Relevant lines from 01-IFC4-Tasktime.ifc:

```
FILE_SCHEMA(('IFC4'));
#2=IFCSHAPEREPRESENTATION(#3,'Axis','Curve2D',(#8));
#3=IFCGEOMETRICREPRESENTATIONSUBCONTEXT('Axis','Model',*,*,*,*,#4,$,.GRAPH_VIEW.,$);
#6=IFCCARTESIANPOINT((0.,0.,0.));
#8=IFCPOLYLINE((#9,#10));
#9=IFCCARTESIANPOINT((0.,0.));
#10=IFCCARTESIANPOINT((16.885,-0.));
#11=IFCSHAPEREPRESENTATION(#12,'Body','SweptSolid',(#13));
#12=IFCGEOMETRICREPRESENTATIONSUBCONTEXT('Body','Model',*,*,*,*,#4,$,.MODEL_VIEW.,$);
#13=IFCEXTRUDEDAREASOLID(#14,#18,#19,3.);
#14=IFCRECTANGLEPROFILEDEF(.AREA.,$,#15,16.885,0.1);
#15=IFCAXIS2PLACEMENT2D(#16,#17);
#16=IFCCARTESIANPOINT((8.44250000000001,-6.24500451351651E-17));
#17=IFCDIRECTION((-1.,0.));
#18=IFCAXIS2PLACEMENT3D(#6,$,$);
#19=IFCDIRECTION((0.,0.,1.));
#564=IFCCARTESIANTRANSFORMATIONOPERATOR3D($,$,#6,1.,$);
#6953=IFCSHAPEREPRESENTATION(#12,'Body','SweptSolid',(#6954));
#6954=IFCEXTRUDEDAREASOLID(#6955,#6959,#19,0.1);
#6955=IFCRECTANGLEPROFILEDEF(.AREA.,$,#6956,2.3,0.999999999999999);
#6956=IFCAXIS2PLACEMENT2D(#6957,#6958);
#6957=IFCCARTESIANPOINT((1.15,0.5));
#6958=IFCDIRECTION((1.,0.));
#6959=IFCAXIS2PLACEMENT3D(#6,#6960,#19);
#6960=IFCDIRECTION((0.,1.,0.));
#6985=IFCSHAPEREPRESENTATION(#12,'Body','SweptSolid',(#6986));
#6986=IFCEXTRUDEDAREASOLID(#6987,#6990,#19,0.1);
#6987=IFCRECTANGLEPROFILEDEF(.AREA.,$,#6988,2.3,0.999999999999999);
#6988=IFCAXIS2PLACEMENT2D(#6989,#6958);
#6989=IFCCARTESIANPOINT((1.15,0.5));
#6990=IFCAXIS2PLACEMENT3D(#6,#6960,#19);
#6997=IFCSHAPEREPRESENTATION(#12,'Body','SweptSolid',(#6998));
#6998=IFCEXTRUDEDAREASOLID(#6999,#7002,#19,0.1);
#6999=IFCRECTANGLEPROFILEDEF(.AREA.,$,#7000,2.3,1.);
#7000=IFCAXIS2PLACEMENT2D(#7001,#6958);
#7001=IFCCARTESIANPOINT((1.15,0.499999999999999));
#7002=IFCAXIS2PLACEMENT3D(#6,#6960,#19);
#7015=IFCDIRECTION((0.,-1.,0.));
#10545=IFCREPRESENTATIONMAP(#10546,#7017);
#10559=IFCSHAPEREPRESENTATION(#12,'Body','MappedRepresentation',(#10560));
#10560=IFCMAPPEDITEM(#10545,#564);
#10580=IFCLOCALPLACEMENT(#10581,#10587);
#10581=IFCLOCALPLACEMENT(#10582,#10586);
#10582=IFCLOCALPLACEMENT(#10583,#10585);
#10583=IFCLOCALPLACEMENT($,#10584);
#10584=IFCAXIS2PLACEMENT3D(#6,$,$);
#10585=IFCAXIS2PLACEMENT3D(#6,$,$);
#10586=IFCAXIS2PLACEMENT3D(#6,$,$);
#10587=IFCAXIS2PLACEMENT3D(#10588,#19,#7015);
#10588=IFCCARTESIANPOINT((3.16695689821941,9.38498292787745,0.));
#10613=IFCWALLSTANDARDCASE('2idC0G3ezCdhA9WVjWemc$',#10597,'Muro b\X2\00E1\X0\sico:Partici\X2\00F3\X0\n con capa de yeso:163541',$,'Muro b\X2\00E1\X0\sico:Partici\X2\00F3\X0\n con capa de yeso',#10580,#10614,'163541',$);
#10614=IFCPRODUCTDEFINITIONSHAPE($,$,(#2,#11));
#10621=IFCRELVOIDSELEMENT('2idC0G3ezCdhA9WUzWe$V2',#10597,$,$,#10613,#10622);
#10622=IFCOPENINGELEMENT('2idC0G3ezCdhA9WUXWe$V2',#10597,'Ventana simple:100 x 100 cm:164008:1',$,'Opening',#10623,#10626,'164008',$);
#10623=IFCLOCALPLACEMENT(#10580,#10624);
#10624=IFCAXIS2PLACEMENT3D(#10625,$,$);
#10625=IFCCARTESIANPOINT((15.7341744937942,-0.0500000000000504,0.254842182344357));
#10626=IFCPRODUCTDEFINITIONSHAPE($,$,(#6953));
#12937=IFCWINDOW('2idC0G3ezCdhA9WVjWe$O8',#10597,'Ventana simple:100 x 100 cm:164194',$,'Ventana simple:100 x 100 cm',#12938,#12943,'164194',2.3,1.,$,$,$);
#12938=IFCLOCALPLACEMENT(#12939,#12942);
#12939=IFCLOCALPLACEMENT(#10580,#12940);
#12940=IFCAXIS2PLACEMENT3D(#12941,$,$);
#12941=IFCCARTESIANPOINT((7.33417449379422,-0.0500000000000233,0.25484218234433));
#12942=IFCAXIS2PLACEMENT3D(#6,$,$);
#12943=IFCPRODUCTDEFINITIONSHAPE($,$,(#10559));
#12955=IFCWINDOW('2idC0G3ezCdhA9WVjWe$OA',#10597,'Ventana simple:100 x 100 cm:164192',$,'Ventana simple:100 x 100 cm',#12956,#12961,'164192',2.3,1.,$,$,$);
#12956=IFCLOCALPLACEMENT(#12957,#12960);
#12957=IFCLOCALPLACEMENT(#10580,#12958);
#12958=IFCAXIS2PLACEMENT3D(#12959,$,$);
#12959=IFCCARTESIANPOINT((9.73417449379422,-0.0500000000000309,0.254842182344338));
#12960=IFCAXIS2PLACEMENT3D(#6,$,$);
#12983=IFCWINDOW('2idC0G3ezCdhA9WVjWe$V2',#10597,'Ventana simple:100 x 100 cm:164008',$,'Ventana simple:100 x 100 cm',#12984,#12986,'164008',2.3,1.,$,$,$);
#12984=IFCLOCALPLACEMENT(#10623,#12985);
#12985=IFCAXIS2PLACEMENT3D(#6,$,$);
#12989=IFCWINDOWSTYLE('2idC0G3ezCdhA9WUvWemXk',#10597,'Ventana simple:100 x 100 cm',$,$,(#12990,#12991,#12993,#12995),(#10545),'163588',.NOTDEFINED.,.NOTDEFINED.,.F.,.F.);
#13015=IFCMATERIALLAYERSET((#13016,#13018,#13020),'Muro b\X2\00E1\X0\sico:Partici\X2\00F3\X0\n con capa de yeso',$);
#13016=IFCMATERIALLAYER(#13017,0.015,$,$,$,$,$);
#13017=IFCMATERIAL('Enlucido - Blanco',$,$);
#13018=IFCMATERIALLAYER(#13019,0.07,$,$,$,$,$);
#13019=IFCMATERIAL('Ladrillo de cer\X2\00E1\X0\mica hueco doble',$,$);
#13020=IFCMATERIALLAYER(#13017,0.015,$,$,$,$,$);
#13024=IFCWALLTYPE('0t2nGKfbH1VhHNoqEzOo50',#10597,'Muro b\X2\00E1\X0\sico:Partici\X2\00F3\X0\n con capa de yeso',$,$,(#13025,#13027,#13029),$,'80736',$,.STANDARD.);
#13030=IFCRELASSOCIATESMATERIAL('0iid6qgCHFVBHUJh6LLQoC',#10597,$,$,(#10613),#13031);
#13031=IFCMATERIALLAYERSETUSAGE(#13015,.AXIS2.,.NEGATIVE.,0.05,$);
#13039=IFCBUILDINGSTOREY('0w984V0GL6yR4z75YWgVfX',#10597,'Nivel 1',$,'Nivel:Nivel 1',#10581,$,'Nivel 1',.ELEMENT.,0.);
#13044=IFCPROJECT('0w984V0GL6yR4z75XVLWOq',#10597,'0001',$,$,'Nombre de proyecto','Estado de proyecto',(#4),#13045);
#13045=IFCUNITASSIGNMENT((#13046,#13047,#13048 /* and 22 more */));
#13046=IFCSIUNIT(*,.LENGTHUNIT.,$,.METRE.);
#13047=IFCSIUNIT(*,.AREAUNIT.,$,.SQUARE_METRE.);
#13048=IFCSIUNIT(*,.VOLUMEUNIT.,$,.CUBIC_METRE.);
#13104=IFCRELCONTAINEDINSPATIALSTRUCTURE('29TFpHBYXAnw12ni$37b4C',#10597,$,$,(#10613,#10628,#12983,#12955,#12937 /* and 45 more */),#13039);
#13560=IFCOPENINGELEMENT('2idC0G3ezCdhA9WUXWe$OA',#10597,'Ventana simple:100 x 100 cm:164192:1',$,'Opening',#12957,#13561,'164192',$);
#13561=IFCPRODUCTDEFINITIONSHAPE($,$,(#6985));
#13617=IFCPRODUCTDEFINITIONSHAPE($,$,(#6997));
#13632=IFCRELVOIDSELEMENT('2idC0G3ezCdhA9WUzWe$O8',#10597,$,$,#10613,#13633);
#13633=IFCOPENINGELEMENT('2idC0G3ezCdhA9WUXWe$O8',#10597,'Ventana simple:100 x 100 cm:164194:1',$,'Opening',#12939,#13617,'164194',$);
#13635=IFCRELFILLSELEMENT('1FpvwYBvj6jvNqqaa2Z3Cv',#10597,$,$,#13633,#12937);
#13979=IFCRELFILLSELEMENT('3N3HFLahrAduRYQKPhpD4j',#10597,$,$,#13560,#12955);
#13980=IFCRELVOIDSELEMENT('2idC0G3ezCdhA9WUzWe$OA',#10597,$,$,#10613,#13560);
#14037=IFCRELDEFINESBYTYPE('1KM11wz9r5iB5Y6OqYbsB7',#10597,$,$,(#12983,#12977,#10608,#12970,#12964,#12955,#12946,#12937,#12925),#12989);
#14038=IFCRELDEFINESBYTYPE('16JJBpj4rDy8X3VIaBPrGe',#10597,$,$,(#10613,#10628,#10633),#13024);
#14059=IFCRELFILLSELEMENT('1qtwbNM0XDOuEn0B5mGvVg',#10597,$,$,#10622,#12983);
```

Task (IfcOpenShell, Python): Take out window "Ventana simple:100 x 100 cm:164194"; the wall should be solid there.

```python
import ifcopenshell
import ifcopenshell.api.feature
import ifcopenshell.api.root
import ifcopenshell.geom
import ifcopenshell.util.shape

model = ifcopenshell.open("01-IFC4-Tasktime.ifc")
settings = ifcopenshell.geom.settings()


def volume(element):
    """Net volume in cubic metres, openings subtracted."""
    shape = ifcopenshell.geom.create_shape(settings, element)
    return ifcopenshell.util.shape.get_volume(shape.geometry)


window = model.by_guid("2idC0G3ezCdhA9WVjWe$O8")
opening = window.FillsVoids[0].RelatingOpeningElement
wall = opening.VoidsElements[0].RelatingBuildingElement
before = volume(wall)

ifcopenshell.api.root.remove_product(model, product=window)
ifcopenshell.api.feature.remove_feature(model, feature=opening)

after = volume(wall)

print(f"wall volume {before:.3f} -> {after:.3f} m3")

model.write("01-IFC4-Tasktime_edited.ifc")
```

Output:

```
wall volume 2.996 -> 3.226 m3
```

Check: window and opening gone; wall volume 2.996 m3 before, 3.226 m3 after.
